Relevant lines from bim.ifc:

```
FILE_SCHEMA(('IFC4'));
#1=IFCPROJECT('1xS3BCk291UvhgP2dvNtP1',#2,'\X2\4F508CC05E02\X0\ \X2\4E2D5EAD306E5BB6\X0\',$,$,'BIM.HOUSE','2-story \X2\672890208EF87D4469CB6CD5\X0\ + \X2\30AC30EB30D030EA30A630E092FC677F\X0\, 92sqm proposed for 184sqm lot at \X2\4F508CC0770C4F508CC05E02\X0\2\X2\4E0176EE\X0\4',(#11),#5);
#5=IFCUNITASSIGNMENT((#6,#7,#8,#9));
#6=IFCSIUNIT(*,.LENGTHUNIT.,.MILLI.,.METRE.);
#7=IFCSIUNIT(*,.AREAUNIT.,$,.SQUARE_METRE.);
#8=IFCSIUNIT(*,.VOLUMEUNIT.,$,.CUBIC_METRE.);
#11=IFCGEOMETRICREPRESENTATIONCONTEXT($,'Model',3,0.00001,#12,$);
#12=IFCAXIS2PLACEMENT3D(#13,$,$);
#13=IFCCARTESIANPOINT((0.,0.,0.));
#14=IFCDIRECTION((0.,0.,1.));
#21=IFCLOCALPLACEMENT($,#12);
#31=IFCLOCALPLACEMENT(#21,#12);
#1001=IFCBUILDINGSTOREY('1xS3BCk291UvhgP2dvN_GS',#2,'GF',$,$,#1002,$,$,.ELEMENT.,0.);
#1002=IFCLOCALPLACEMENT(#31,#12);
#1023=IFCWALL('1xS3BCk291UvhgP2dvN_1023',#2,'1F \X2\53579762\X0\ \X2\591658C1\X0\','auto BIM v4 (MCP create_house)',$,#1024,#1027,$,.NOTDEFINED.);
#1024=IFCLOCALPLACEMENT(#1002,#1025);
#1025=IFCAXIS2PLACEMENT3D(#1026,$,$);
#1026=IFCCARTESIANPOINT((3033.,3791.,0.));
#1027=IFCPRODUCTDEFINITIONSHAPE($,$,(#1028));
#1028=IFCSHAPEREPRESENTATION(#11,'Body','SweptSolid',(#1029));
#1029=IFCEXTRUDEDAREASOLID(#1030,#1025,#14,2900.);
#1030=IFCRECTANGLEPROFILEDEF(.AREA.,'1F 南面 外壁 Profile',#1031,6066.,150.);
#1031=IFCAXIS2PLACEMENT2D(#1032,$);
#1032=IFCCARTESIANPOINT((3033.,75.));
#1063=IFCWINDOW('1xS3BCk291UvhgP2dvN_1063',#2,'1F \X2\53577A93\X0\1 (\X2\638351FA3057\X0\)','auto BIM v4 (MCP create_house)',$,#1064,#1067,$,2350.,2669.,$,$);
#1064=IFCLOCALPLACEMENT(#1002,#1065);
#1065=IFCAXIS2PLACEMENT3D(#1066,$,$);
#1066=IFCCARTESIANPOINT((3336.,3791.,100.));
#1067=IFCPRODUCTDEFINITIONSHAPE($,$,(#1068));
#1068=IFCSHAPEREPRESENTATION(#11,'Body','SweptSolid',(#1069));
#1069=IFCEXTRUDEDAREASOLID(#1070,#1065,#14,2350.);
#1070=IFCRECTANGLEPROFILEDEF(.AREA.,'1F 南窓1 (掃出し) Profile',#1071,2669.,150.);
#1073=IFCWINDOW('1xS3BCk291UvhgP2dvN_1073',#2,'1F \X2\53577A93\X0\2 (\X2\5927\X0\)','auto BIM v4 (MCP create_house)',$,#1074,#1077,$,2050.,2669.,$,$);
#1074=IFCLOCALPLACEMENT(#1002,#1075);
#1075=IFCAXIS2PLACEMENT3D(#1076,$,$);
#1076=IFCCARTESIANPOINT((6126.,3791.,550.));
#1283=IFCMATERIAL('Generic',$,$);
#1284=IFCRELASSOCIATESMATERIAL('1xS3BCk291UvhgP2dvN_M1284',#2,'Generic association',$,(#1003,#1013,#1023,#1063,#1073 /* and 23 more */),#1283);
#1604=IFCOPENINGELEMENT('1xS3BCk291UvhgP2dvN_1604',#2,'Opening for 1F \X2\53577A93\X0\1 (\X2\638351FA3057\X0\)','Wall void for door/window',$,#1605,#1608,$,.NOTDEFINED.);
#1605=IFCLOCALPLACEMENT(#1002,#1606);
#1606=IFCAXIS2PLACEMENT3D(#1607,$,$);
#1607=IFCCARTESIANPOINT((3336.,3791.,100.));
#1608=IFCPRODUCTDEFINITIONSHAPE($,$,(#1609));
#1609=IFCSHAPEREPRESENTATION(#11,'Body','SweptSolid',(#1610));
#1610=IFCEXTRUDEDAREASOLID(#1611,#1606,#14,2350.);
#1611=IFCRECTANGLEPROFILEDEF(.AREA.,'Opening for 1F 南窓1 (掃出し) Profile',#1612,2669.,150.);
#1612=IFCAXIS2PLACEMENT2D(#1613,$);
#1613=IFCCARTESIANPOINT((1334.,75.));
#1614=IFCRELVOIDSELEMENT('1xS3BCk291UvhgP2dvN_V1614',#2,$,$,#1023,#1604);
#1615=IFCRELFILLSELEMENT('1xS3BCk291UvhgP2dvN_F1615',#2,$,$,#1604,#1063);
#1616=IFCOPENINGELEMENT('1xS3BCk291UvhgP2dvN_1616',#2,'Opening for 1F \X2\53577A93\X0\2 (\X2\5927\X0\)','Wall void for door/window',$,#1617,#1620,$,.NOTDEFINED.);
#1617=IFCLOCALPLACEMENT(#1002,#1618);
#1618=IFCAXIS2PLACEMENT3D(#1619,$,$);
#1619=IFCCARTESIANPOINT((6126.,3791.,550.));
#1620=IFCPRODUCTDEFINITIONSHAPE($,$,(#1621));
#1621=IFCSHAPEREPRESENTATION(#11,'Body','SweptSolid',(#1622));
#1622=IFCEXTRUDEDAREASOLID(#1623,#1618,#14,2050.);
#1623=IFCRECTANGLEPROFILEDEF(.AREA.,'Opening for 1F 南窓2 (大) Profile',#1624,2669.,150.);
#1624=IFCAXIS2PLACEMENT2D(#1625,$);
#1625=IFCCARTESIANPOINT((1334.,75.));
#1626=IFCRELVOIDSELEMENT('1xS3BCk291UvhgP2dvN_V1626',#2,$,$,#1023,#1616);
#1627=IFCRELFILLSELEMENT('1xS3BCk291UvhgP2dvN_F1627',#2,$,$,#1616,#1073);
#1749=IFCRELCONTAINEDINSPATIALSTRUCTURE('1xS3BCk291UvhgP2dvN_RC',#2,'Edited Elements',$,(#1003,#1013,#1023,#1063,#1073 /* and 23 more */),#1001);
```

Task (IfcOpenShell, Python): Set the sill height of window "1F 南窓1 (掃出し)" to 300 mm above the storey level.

```python
import numpy as np
import ifcopenshell
import ifcopenshell.api.geometry
import ifcopenshell.geom
import ifcopenshell.util.element
import ifcopenshell.util.placement
import ifcopenshell.util.shape
import ifcopenshell.util.unit

model = ifcopenshell.open("bim.ifc")
unit_scale = ifcopenshell.util.unit.calculate_unit_scale(model)

window = model.by_guid("1xS3BCk291UvhgP2dvN_1063")
opening = window.FillsVoids[0].RelatingOpeningElement
storey = ifcopenshell.util.element.get_container(window, ifc_class="IfcBuildingStorey")
level = ifcopenshell.util.placement.get_local_placement(storey.ObjectPlacement)[2, 3]

# The opening's origin need not be at the sill, so measure its lowest point.
shape = ifcopenshell.geom.create_shape(ifcopenshell.geom.settings(), opening)
bottom = ifcopenshell.util.shape.get_shape_bottom_elevation(shape, shape.geometry) / unit_scale
dz = level + 0.3 / unit_scale - bottom

shift = np.array([0.0, 0.0, dz])
# The window is not placed relative to its opening, so move both.
for product in (opening, window):
    matrix = ifcopenshell.util.placement.get_local_placement(product.ObjectPlacement)
    matrix[:3, 3] += shift
    ifcopenshell.api.geometry.edit_object_placement(model, product=product, matrix=matrix, is_si=False)

print(f"moved by {dz * unit_scale:+.3f} m")

model.write("bim_updated.ifc")
```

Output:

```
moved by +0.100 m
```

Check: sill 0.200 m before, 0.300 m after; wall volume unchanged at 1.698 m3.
